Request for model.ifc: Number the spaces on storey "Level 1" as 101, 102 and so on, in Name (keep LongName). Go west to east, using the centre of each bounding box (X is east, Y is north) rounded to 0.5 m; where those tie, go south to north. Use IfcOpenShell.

First a look at what the model holds.

```python
import ifcopenshell
import ifcopenshell.util.element
import ifcopenshell.util.placement

model = ifcopenshell.open("model.ifc")
print(model.schema)
storey = next(s for s in model.by_type("IfcBuildingStorey") if s.Name == "Level 1")
spaces = [e for e in ifcopenshell.util.element.get_decomposition(storey) if e.is_a("IfcSpace")]
for e in sorted(spaces, key=lambda e: e.id()):
    origin = ifcopenshell.util.placement.get_local_placement(e.ObjectPlacement)[:3, 3]
    print(e.id(), e.Name, e.LongName, origin.round(2) + 0.0, sep=" | ")
```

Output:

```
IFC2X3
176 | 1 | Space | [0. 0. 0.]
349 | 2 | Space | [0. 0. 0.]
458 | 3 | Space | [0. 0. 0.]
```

```python
import ifcopenshell
import ifcopenshell.geom
import ifcopenshell.util.element
import ifcopenshell.util.shape

model = ifcopenshell.open("model.ifc")
settings = ifcopenshell.geom.settings()
settings.set("use-world-coords", True)


def centre(element):
    shape = ifcopenshell.geom.create_shape(settings, element)
    return ifcopenshell.util.shape.get_bbox_centroid(shape.geometry)


storey = next(s for s in model.by_type("IfcBuildingStorey") if s.Name == "Level 1")
spaces = [e for e in ifcopenshell.util.element.get_decomposition(storey) if e.is_a("IfcSpace")]

# Insertion points can sit at a corner or the storey origin, so sort by the geometry (in metres).
centres = {e: centre(e) for e in spaces}
spaces.sort(key=lambda e: (round(centres[e][0] / 0.5), centres[e][1]))

for i, e in enumerate(spaces, start=1):
    number = f"1{i:02d}"
    e.Name = number
    print(e.id(), number)

model.write("model_v2.ifc")
```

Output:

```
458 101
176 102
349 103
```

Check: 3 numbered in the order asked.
